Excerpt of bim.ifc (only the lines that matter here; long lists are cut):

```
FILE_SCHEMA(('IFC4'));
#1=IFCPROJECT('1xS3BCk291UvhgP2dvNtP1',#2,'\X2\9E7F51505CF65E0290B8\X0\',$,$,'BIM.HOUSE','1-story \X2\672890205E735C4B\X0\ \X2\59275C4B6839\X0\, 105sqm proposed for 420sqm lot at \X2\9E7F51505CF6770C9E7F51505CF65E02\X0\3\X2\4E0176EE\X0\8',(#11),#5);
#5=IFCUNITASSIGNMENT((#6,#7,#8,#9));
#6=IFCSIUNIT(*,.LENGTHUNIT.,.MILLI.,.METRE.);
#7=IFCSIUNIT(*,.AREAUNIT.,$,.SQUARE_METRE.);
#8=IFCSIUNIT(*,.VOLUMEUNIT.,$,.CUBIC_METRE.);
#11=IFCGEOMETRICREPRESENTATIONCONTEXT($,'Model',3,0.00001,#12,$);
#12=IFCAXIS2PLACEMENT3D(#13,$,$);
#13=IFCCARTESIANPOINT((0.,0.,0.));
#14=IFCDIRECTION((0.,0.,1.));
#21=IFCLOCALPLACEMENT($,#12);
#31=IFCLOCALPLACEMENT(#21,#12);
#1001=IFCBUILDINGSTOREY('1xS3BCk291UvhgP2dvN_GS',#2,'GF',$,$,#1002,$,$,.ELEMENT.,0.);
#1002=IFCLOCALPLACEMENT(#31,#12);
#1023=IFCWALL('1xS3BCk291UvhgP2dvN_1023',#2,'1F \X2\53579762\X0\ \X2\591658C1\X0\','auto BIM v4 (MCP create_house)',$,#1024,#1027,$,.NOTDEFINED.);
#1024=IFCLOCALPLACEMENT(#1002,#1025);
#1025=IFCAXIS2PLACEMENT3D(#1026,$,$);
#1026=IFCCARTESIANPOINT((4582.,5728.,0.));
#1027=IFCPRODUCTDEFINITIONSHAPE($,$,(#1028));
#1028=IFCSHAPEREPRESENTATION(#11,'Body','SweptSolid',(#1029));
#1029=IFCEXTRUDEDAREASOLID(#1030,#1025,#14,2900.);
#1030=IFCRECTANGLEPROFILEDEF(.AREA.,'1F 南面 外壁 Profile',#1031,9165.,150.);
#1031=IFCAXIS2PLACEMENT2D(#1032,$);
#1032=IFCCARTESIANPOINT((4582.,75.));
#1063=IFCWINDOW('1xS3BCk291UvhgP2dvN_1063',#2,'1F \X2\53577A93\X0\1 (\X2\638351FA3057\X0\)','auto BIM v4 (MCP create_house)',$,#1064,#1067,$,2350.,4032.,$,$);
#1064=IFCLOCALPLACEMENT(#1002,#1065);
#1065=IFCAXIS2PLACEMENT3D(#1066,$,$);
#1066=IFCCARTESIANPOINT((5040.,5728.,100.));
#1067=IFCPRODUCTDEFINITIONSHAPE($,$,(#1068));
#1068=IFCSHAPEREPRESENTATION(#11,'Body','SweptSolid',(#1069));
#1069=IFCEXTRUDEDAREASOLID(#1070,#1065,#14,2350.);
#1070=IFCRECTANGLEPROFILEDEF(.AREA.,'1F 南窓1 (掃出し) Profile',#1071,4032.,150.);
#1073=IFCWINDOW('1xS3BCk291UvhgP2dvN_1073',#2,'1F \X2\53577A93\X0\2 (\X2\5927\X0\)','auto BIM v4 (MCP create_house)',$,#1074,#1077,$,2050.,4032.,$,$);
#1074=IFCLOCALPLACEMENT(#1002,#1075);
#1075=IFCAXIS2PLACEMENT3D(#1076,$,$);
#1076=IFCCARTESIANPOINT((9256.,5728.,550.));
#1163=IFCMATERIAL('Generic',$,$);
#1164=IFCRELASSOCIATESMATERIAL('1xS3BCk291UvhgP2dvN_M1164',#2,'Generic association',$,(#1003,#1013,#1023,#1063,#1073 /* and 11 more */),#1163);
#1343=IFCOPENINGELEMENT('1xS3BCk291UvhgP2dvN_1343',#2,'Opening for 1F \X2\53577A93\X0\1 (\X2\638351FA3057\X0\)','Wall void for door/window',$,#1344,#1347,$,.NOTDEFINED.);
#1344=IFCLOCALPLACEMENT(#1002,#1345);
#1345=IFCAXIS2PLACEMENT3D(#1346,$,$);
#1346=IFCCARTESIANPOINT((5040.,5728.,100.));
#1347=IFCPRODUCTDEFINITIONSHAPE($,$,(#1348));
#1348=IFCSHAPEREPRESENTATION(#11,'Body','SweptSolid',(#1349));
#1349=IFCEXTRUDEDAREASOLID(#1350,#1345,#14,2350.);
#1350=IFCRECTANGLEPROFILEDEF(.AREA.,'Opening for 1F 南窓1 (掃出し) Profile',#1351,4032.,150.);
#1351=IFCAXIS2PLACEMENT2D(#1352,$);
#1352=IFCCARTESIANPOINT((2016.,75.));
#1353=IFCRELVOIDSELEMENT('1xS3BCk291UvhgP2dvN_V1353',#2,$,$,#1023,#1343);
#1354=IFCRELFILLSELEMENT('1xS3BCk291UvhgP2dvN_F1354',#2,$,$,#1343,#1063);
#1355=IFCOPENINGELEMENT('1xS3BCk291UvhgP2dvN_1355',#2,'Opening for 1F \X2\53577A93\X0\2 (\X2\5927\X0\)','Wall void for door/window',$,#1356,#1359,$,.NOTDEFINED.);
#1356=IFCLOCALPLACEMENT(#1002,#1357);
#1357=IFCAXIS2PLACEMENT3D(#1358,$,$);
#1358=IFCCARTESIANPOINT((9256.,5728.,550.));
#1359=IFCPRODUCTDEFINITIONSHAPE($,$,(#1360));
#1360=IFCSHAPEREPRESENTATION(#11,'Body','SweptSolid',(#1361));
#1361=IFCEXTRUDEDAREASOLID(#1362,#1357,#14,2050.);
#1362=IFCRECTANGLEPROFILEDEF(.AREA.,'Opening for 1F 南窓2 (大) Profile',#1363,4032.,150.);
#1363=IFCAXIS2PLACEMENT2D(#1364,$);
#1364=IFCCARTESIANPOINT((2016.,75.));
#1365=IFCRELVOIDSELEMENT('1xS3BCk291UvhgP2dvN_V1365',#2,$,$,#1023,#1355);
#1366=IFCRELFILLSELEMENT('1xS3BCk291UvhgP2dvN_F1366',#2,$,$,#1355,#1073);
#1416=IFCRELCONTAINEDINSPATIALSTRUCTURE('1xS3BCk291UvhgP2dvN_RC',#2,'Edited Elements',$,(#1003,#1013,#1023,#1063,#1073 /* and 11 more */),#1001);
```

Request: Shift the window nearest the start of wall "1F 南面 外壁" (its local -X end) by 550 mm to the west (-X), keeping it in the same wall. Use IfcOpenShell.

```python
import ifcopenshell
import ifcopenshell.api.geometry
import ifcopenshell.util.placement

model = ifcopenshell.open("bim.ifc")

window = model.by_id(1063)
opening = window.FillsVoids[0].RelatingOpeningElement
wall = opening.VoidsElements[0].RelatingBuildingElement

wall_matrix = ifcopenshell.util.placement.get_local_placement(wall.ObjectPlacement)
shift = wall_matrix[:3, 0] * -550.0
before = ifcopenshell.util.placement.get_local_placement(window.ObjectPlacement)[:3, 3].copy()

# The window is not placed relative to its opening, so move both.
for product in (opening, window):
    matrix = ifcopenshell.util.placement.get_local_placement(product.ObjectPlacement)
    matrix[:3, 3] += shift
    ifcopenshell.api.geometry.edit_object_placement(model, product=product, matrix=matrix, is_si=False)

after = ifcopenshell.util.placement.get_local_placement(window.ObjectPlacement)[:3, 3]
print("window moved by", (after - before).round(3) + 0.0)

model.write("bim_updated.ifc")
```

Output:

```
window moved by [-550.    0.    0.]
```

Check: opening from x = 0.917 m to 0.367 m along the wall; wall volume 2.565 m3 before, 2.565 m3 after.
